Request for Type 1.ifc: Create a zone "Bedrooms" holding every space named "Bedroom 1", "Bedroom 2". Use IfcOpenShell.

First a look at what the model holds.

```python
import ifcopenshell

model = ifcopenshell.open("Type 1.ifc")
print(model.schema)
seen = {}
for space in model.by_type("IfcSpace"):
    seen[space.LongName] = seen.get(space.LongName, 0) + 1
for name, count in sorted(seen.items(), key=str):
    print(count, "x", name)
print("zones:", [z.Name for z in model.by_type("IfcZone")][:20])
```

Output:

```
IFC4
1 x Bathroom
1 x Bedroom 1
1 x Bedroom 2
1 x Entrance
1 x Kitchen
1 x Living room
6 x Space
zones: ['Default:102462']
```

```python
import ifcopenshell
import ifcopenshell.api.group
import ifcopenshell.api.root

model = ifcopenshell.open("Type 1.ifc")

names = {"Bedroom 1", "Bedroom 2"}
spaces = [s for s in model.by_type("IfcSpace") if s.LongName in names]

zone = ifcopenshell.api.root.create_entity(model, ifc_class="IfcZone", name="Bedrooms")
ifcopenshell.api.group.assign_group(model, products=spaces, group=zone)
print(len(spaces), "spaces in", zone.Name)

model.write("Type 1_updated.ifc")
```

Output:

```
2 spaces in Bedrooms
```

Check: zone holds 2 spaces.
